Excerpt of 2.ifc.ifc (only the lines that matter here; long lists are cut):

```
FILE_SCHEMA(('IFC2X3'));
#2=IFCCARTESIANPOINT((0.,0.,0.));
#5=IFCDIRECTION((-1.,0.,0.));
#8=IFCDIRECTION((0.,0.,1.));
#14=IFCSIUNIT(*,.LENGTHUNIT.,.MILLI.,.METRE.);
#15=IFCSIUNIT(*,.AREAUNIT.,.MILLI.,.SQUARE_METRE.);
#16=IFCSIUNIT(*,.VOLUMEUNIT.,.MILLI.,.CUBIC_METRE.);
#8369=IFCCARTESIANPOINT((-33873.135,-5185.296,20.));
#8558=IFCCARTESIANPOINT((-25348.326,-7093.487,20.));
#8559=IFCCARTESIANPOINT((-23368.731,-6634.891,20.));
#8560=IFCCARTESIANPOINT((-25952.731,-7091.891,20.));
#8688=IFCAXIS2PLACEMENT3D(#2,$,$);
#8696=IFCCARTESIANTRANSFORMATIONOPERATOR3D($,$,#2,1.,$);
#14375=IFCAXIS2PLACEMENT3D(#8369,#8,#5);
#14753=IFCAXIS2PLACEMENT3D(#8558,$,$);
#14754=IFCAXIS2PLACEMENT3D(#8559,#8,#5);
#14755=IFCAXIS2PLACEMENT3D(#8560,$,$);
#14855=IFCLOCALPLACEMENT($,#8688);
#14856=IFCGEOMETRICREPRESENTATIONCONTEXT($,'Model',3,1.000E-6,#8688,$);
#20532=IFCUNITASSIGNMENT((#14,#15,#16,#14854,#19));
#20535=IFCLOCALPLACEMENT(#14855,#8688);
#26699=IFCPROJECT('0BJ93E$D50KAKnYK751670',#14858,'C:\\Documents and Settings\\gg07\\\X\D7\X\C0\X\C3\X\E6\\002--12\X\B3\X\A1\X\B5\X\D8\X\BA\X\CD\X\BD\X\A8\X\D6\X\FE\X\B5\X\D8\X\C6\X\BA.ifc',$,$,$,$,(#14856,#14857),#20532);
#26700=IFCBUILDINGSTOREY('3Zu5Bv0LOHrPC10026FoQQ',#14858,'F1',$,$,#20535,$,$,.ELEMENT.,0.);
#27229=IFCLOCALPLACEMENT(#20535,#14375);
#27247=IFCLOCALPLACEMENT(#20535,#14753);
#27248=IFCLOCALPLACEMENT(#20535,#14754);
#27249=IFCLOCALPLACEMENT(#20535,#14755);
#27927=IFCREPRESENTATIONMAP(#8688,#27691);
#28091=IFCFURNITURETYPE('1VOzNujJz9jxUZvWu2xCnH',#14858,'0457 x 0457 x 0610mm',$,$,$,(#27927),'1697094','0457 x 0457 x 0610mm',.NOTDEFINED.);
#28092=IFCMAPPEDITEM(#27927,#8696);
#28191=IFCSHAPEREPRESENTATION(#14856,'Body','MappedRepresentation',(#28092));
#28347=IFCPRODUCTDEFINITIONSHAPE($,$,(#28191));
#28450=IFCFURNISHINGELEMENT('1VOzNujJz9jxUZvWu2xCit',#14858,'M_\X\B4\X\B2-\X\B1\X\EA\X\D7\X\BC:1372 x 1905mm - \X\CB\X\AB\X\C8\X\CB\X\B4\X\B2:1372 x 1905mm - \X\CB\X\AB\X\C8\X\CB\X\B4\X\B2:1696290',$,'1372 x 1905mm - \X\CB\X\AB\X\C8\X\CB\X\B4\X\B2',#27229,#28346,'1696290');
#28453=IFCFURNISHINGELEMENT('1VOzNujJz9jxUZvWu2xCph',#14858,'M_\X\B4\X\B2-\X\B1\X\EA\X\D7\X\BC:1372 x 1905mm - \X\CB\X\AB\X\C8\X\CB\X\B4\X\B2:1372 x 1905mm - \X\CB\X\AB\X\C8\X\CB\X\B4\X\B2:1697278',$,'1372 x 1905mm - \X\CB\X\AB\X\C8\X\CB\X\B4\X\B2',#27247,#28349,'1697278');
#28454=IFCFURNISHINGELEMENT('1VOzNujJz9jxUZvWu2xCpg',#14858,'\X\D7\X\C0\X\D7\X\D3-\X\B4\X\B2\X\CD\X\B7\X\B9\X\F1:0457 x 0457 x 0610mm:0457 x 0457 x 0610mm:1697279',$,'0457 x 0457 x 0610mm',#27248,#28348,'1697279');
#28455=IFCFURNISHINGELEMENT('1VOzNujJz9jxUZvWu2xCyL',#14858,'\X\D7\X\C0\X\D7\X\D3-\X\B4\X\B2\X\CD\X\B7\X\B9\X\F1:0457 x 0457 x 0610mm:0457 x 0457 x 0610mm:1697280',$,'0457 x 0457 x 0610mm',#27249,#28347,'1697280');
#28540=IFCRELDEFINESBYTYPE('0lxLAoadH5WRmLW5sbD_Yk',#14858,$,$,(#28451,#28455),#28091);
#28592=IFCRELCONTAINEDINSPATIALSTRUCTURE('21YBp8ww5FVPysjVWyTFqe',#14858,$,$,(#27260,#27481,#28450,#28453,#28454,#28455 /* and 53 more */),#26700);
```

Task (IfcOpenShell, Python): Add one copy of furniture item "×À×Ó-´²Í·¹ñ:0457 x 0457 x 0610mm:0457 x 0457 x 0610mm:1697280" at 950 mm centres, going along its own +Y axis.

```python
import ifcopenshell
import ifcopenshell.api.geometry
import ifcopenshell.api.root
import ifcopenshell.util.element
import ifcopenshell.util.placement
import ifcopenshell.util.unit

model = ifcopenshell.open("2.ifc.ifc")
unit_scale = ifcopenshell.util.unit.calculate_unit_scale(model)


def reuse_history(source, copy):
    """copy_class also copies each property set's owner history, people and application; keep the originals."""
    for rel in copy.IsDefinedBy:
        if rel.is_a("IfcRelDefinesByProperties") and (history := rel.RelatingPropertyDefinition.OwnerHistory):
            rel.RelatingPropertyDefinition.OwnerHistory = source.OwnerHistory
            ifcopenshell.util.element.remove_deep2(model, history)


source = model.by_id(28455)
base = ifcopenshell.util.placement.get_local_placement(source.ObjectPlacement)
step = base[:3, 1] * 0.95 / unit_scale

for i in range(1, 2):
    copy = ifcopenshell.api.root.copy_class(model, product=source)
    copy.Representation = ifcopenshell.util.element.copy_deep(
        model, source.Representation, exclude=["IfcGeometricRepresentationContext", "IfcRepresentationMap"]
    )
    copy.Name = "×À×Ó-´²Í·¹ñ:0457 x 0457 x 0610mm:0457 x 0457 x 0610mm"
    copy.Tag = None
    reuse_history(source, copy)
    matrix = base.copy()
    matrix[:3, 3] += i * step
    print("added at", matrix[:3, 3].round(3) + 0.0)
    ifcopenshell.api.geometry.edit_object_placement(model, product=copy, matrix=matrix, is_si=False)

model.write("2.ifc_v2.ifc")
```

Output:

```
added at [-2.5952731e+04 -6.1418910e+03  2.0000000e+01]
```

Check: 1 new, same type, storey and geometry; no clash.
